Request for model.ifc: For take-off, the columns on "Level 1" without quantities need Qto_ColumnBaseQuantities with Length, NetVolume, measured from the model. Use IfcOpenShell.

First a look at what the model holds.

```python
import ifcopenshell
import ifcopenshell.util.element
import ifcopenshell.util.unit

model = ifcopenshell.open("model.ifc")
print(model.schema)
for unit_type in ("LENGTHUNIT", "AREAUNIT", "VOLUMEUNIT"):
    print(unit_type, ifcopenshell.util.unit.calculate_unit_scale(model, unit_type))
storey = next(s for s in model.by_type("IfcBuildingStorey") if s.Name == "Level 1")
columns = [e for e in ifcopenshell.util.element.get_decomposition(storey) if e.is_a("IfcColumn")]
for e in sorted(columns, key=lambda e: e.id()):
    print(e.id(), e.is_a(), e.Name, list(ifcopenshell.util.element.get_psets(e, qtos_only=True)), sep=" | ")
```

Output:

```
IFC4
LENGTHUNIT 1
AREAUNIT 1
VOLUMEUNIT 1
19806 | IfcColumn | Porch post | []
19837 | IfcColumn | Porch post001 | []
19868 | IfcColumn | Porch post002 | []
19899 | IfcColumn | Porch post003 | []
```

```python
import ifcopenshell
import ifcopenshell.api.pset
import ifcopenshell.geom
import ifcopenshell.util.element
import ifcopenshell.util.shape
import ifcopenshell.util.unit

model = ifcopenshell.open("model.ifc")
unit_scale = ifcopenshell.util.unit.calculate_unit_scale(model)
volume_scale = ifcopenshell.util.unit.calculate_unit_scale(model, "VOLUMEUNIT")
settings = ifcopenshell.geom.settings()

storey = next(s for s in model.by_type("IfcBuildingStorey") if s.Name == "Level 1")
columns = [e for e in ifcopenshell.util.element.get_decomposition(storey) if e.is_a("IfcColumn")]

for e in sorted(columns, key=lambda e: e.id()):
    if ifcopenshell.util.element.get_psets(e, qtos_only=True, should_inherit=False):
        continue
    # Geometry comes back in metres, in the element's own axes.
    shape = ifcopenshell.geom.create_shape(settings, e)
    values = {
        "Length": ifcopenshell.util.shape.get_z(shape.geometry) / unit_scale,
        "NetVolume": ifcopenshell.util.shape.get_volume(shape.geometry) / volume_scale,
    }
    qto = ifcopenshell.api.pset.add_qto(model, product=e, name="Qto_ColumnBaseQuantities")
    ifcopenshell.api.pset.edit_qto(model, qto=qto, properties=values)
    print(e.id(), {k: round(v, 3) for k, v in values.items()})

model.write("model_v2.ifc")
```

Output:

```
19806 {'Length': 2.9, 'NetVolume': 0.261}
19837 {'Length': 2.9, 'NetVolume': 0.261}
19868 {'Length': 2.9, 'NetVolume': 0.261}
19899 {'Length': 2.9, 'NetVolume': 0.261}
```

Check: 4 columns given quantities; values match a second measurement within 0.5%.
